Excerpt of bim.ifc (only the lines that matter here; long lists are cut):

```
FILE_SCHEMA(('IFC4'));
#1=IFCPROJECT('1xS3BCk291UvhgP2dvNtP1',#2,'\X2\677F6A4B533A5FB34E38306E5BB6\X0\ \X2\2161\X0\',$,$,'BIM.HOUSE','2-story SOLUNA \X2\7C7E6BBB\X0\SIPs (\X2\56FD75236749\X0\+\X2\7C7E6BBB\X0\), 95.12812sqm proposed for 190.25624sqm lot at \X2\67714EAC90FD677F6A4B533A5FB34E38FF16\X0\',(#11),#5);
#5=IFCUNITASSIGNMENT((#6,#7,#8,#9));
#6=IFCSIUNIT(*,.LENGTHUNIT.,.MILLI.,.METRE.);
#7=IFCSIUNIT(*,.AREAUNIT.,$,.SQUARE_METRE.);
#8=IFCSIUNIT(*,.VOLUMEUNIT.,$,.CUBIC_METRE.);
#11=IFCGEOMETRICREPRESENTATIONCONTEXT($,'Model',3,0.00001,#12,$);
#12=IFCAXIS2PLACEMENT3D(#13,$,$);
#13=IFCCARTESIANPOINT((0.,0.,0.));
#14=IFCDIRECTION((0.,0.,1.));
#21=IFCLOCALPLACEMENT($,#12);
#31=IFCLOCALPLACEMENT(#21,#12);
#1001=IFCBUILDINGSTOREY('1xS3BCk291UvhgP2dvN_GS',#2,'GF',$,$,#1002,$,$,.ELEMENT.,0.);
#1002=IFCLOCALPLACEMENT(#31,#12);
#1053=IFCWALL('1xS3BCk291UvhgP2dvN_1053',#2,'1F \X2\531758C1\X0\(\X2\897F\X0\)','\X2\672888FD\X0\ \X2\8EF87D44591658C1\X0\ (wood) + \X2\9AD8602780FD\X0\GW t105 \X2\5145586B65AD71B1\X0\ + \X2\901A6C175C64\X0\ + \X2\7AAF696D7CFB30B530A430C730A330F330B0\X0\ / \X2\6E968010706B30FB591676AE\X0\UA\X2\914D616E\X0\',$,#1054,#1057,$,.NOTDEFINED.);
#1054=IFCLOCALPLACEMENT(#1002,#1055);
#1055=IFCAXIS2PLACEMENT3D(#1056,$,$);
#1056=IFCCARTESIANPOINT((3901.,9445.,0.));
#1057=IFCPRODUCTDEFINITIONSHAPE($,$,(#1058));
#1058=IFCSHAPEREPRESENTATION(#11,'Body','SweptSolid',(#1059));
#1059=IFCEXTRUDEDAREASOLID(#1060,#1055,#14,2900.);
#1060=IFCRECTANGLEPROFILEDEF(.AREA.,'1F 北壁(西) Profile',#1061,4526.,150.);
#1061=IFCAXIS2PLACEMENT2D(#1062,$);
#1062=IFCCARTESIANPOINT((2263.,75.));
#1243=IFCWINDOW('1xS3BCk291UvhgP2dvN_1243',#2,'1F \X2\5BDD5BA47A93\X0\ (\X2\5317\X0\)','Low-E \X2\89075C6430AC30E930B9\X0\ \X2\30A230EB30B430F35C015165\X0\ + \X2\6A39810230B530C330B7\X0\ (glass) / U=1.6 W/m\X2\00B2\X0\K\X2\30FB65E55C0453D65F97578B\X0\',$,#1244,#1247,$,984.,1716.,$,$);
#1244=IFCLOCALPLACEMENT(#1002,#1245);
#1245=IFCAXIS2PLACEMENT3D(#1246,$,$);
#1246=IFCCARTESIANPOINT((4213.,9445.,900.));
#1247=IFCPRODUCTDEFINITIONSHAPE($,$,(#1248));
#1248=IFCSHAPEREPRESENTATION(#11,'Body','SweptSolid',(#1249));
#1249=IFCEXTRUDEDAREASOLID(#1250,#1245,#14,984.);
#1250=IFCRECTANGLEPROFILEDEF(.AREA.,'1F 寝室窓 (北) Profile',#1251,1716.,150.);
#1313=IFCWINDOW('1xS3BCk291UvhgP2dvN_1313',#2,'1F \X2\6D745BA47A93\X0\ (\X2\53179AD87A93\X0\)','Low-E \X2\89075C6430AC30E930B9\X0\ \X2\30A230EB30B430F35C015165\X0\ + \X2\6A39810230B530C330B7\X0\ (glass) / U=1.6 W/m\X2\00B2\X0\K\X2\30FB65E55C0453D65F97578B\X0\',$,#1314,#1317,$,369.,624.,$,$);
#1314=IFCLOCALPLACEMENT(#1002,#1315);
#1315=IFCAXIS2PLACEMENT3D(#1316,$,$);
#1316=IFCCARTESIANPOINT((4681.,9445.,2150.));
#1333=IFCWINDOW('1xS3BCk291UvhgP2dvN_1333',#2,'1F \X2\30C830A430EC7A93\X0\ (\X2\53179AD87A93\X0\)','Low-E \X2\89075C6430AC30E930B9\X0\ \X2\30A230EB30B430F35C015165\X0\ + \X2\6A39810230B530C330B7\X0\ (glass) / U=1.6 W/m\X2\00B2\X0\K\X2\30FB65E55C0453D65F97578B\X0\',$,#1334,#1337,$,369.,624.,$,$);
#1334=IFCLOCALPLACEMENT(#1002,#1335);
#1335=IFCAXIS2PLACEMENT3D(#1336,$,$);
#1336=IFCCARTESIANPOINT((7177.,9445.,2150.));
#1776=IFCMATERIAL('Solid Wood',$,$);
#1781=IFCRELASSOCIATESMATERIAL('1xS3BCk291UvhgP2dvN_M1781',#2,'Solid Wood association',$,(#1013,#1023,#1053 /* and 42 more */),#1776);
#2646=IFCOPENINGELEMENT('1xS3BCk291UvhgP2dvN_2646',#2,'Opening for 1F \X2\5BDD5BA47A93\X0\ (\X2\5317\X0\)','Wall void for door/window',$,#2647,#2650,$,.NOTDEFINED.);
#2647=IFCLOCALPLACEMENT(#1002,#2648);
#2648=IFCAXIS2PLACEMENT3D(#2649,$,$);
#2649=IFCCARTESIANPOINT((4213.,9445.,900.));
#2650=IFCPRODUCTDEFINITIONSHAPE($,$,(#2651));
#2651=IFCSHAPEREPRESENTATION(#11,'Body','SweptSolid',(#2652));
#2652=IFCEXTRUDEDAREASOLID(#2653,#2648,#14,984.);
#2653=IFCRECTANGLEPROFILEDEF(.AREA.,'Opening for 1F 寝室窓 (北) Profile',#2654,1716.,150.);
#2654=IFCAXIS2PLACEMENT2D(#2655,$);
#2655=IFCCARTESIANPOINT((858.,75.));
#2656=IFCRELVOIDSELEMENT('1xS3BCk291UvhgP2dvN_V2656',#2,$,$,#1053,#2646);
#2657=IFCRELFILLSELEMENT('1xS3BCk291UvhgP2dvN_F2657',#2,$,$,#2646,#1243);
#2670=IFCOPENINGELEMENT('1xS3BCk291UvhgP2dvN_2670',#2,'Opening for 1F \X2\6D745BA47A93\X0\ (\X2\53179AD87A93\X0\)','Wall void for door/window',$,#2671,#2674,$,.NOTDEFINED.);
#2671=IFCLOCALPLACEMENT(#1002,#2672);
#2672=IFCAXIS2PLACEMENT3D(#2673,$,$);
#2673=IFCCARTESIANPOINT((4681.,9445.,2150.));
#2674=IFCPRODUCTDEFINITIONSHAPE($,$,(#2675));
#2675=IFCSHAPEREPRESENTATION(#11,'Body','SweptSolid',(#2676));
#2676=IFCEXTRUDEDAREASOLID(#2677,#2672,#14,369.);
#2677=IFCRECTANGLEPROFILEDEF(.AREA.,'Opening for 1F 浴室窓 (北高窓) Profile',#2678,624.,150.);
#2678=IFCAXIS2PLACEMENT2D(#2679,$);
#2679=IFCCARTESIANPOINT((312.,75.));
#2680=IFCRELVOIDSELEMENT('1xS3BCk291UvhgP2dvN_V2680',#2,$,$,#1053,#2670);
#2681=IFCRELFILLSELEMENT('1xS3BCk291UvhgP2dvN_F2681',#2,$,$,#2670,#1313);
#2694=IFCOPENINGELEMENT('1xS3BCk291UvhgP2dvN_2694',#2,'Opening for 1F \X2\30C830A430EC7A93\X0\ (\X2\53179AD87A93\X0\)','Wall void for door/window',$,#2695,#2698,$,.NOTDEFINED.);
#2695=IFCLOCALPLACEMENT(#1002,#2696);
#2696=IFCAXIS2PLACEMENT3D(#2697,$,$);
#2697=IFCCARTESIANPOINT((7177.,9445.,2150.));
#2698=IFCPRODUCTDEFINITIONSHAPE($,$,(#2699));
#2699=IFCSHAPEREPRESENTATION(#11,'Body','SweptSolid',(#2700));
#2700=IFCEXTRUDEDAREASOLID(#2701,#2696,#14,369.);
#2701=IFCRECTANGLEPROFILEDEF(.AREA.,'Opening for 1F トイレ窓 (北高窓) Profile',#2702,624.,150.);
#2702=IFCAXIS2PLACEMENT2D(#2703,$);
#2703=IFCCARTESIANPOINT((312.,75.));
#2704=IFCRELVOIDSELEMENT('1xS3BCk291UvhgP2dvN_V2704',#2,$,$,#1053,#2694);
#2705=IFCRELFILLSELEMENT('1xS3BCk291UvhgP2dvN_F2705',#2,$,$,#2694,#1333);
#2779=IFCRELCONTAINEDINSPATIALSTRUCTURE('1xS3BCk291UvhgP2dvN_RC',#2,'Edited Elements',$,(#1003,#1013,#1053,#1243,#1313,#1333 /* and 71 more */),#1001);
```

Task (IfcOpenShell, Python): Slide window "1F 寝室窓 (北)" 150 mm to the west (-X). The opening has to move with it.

```python
import ifcopenshell
import ifcopenshell.api.geometry
import ifcopenshell.util.placement

model = ifcopenshell.open("bim.ifc")

window = model.by_guid("1xS3BCk291UvhgP2dvN_1243")
opening = window.FillsVoids[0].RelatingOpeningElement
wall = opening.VoidsElements[0].RelatingBuildingElement

wall_matrix = ifcopenshell.util.placement.get_local_placement(wall.ObjectPlacement)
shift = wall_matrix[:3, 0] * -150.0
before = ifcopenshell.util.placement.get_local_placement(window.ObjectPlacement)[:3, 3].copy()

# The window is not placed relative to its opening, so move both.
for product in (opening, window):
    matrix = ifcopenshell.util.placement.get_local_placement(product.ObjectPlacement)
    matrix[:3, 3] += shift
    ifcopenshell.api.geometry.edit_object_placement(model, product=product, matrix=matrix, is_si=False)

after = ifcopenshell.util.placement.get_local_placement(window.ObjectPlacement)[:3, 3]
print("window moved by", (after - before).round(3) + 0.0)

model.write("bim_updated.ifc")
```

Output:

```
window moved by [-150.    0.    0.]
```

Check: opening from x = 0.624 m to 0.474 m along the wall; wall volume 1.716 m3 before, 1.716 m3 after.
